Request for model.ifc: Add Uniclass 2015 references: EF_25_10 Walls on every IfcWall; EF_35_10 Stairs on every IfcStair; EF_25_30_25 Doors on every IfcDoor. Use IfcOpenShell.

First a look at what the model holds.

```python
import ifcopenshell

model = ifcopenshell.open("model.ifc")
print(model.schema)
print("classifications:", [c.Name for c in model.by_type("IfcClassification")])
for ifc_class in ("IfcDoor", "IfcRoof", "IfcStair", "IfcWall", "IfcWindow"):
    print(ifc_class, len(model.by_type(ifc_class)))
```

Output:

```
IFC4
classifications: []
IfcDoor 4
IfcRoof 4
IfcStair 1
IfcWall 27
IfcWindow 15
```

```python
import ifcopenshell
import ifcopenshell.api.classification

model = ifcopenshell.open("model.ifc")

system = ifcopenshell.api.classification.add_classification(model, classification="Uniclass 2015")

codes = {
    "IfcWall": ("EF_25_10", "Walls"),
    "IfcStair": ("EF_35_10", "Stairs"),
    "IfcDoor": ("EF_25_30_25", "Doors"),
}
for ifc_class, (code, name) in codes.items():
    products = model.by_type(ifc_class)
    ifcopenshell.api.classification.add_reference(
        model, products=products, classification=system, identification=code, name=name
    )
    print(code, len(products))

model.write("model_updated.ifc")
```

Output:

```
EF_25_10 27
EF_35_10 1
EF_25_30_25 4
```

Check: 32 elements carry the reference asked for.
